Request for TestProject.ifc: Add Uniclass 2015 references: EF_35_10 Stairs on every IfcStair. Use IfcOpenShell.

First a look at what the model holds.

```python
import ifcopenshell

model = ifcopenshell.open("TestProject.ifc")
print(model.schema)
print("classifications:", [c.Name for c in model.by_type("IfcClassification")])
for ifc_class in ("IfcDoor", "IfcRoof", "IfcStair", "IfcWall", "IfcWindow"):
    print(ifc_class, len(model.by_type(ifc_class)))
```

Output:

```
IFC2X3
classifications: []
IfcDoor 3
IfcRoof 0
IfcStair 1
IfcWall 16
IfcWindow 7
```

```python
import ifcopenshell
import ifcopenshell.api.classification

model = ifcopenshell.open("TestProject.ifc")

# IFC2X3 requires Source and Edition and has no link from the project to the system.
system = model.create_entity("IfcClassification", Source="NBS", Edition="2015", Name="Uniclass 2015")

codes = {
    "IfcStair": ("EF_35_10", "Stairs"),
}
for ifc_class, (code, name) in codes.items():
    products = model.by_type(ifc_class)
    ifcopenshell.api.classification.add_reference(
        model, products=products, classification=system, identification=code, name=name
    )
    print(code, len(products))

model.write("TestProject_updated.ifc")
```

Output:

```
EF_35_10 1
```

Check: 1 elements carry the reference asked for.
